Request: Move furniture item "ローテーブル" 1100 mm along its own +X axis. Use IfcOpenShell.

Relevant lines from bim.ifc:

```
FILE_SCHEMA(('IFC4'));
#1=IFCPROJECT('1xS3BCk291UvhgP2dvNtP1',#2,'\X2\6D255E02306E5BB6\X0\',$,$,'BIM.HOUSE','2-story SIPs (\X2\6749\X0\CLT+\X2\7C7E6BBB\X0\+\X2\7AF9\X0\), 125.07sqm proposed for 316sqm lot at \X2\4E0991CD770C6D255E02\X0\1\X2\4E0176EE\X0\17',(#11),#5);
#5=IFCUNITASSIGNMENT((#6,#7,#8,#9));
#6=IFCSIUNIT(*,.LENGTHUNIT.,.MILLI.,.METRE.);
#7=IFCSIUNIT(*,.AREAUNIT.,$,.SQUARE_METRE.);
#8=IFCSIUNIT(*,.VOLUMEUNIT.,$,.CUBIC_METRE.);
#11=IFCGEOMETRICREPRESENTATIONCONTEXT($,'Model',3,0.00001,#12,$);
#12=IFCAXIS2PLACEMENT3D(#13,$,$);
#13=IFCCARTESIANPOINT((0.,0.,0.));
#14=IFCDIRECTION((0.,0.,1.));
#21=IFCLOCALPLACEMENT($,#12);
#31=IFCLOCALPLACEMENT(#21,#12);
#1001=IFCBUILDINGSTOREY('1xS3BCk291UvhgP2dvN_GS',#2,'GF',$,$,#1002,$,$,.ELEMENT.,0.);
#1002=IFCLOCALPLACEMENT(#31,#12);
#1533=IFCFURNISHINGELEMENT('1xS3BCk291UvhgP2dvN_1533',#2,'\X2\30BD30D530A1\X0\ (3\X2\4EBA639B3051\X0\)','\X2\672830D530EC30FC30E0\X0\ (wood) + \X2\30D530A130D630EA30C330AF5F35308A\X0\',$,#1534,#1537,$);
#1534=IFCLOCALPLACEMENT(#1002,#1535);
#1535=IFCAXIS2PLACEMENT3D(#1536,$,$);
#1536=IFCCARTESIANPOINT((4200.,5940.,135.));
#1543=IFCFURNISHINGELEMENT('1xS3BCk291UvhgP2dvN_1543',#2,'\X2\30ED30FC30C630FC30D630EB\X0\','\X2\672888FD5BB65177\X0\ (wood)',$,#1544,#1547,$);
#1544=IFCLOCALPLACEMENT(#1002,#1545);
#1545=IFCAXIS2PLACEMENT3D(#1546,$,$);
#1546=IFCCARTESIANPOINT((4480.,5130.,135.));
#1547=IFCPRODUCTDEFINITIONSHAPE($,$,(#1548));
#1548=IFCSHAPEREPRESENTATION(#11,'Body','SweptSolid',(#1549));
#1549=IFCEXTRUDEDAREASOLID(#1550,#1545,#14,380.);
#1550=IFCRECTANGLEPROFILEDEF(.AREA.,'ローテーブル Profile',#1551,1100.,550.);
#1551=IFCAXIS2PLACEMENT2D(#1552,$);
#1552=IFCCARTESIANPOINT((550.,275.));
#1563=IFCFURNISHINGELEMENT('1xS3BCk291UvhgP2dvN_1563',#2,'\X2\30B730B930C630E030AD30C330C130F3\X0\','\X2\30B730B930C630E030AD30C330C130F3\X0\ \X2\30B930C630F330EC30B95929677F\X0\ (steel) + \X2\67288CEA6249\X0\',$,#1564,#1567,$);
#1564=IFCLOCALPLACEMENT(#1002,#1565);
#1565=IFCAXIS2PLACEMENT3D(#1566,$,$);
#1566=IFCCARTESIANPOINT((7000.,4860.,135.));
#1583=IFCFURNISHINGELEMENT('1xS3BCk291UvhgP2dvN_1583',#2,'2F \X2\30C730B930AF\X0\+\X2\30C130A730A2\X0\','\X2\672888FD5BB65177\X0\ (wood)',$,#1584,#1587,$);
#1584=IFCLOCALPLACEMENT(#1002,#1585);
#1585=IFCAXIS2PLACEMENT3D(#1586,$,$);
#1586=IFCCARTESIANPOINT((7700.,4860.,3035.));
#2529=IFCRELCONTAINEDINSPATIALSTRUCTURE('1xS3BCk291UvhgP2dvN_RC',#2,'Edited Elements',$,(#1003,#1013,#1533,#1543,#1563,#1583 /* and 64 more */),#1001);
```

```python
import ifcopenshell
import ifcopenshell.api.geometry
import ifcopenshell.util.placement
import ifcopenshell.util.unit

model = ifcopenshell.open("bim.ifc")
unit_scale = ifcopenshell.util.unit.calculate_unit_scale(model)

item = model.by_guid("1xS3BCk291UvhgP2dvN_1543")
matrix = ifcopenshell.util.placement.get_local_placement(item.ObjectPlacement)
matrix[:3, 3] += matrix[:3, 0] * 1.1 / unit_scale
ifcopenshell.api.geometry.edit_object_placement(model, product=item, matrix=matrix, is_si=False)

print(ifcopenshell.util.placement.get_local_placement(item.ObjectPlacement).round(3) + 0.0)

model.write("bim_updated.ifc")
```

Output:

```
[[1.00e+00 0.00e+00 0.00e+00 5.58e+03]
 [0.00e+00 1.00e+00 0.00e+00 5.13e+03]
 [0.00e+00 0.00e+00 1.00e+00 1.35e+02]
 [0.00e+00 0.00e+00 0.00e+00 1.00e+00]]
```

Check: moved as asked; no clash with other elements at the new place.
